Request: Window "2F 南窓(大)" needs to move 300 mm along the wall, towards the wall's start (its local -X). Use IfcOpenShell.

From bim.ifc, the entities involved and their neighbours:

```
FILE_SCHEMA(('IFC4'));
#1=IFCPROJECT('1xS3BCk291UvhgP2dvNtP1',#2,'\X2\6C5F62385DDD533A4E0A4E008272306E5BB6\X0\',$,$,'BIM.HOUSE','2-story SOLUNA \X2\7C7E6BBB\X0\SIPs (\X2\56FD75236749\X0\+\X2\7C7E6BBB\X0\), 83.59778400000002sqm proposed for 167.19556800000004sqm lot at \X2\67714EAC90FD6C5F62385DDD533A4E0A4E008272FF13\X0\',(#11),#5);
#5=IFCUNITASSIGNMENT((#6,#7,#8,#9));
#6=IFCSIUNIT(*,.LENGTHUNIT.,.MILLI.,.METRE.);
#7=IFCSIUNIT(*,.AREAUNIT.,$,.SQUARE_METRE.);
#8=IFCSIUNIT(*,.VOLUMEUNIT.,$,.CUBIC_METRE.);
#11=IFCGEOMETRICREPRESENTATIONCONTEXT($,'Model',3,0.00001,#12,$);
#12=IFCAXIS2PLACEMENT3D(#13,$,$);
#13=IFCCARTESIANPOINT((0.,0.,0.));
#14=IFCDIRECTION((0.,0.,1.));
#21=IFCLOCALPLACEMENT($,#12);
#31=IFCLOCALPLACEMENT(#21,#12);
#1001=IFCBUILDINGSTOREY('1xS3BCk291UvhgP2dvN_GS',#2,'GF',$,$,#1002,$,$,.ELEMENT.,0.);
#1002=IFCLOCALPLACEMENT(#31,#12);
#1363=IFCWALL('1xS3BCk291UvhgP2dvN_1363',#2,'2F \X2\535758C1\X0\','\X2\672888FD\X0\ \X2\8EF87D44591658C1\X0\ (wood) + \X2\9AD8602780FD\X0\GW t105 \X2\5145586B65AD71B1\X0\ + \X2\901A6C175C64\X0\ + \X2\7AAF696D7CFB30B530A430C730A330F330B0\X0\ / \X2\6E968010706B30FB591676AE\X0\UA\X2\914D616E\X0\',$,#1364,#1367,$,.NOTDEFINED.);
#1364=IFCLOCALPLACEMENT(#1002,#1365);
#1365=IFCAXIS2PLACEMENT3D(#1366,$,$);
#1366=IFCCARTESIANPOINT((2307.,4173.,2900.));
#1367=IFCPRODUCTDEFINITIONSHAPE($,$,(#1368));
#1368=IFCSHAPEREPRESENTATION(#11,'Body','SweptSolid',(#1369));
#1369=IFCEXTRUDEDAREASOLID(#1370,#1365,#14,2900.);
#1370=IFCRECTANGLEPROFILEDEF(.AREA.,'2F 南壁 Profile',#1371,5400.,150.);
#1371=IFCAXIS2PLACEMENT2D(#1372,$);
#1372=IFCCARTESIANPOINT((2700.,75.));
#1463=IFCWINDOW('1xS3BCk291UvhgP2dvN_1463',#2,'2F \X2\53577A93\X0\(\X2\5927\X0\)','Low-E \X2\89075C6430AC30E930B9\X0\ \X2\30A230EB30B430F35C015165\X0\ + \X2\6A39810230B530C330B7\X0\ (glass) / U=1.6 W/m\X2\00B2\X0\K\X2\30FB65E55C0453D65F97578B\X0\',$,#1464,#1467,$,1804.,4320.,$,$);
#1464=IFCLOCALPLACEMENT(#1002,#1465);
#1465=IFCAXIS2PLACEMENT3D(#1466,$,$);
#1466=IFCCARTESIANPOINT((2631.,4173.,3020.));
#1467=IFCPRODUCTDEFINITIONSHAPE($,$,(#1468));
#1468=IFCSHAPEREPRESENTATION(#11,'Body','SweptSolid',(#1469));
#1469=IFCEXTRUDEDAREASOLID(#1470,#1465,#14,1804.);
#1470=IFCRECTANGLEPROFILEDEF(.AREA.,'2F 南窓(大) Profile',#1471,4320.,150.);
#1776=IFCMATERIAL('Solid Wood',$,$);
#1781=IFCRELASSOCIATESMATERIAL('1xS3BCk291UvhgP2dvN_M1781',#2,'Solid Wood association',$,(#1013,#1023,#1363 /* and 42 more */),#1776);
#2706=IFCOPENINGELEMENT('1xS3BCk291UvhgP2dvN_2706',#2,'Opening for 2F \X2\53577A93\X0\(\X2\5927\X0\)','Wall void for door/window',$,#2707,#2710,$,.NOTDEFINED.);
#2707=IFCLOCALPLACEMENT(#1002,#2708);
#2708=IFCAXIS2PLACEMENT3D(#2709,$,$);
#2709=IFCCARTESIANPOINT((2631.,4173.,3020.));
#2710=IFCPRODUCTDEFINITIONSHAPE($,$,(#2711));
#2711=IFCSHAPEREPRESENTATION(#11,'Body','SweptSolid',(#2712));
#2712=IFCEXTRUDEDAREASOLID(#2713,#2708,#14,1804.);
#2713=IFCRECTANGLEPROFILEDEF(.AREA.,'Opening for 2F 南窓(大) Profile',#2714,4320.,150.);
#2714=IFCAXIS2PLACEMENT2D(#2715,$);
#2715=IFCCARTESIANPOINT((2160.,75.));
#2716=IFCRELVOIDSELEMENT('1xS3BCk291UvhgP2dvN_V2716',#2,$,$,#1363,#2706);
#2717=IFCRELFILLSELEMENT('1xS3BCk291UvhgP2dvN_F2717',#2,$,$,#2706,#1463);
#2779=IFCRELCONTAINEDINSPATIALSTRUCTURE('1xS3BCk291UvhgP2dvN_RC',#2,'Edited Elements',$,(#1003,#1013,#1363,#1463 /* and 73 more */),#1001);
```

```python
import ifcopenshell
import ifcopenshell.api.geometry
import ifcopenshell.util.placement
import ifcopenshell.util.unit

model = ifcopenshell.open("bim.ifc")
unit_scale = ifcopenshell.util.unit.calculate_unit_scale(model)

window = model.by_guid("1xS3BCk291UvhgP2dvN_1463")
opening = window.FillsVoids[0].RelatingOpeningElement
wall = opening.VoidsElements[0].RelatingBuildingElement

wall_matrix = ifcopenshell.util.placement.get_local_placement(wall.ObjectPlacement)
shift = wall_matrix[:3, 0] * -0.3 / unit_scale
before = ifcopenshell.util.placement.get_local_placement(window.ObjectPlacement)[:3, 3].copy()

# The window is not placed relative to its opening, so move both.
for product in (opening, window):
    matrix = ifcopenshell.util.placement.get_local_placement(product.ObjectPlacement)
    matrix[:3, 3] += shift
    ifcopenshell.api.geometry.edit_object_placement(model, product=product, matrix=matrix, is_si=False)

after = ifcopenshell.util.placement.get_local_placement(window.ObjectPlacement)[:3, 3]
print("window moved by", (after - before).round(3) + 0.0)

model.write("bim_updated.ifc")
```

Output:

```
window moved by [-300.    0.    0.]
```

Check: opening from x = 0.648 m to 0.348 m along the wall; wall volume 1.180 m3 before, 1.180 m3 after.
